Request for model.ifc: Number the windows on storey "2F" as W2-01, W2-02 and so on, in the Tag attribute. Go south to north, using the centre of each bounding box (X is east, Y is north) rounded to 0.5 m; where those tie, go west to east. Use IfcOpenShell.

First a look at what the model holds.

```python
import ifcopenshell
import ifcopenshell.util.element
import ifcopenshell.util.placement

model = ifcopenshell.open("model.ifc")
print(model.schema)
storey = next(s for s in model.by_type("IfcBuildingStorey") if s.Name == "2F")
windows = [e for e in ifcopenshell.util.element.get_decomposition(storey) if e.is_a("IfcWindow")]
for e in sorted(windows, key=lambda e: e.id()):
    origin = ifcopenshell.util.placement.get_local_placement(e.ObjectPlacement)[:3, 3]
    print(e.id(), e.Tag, e.Name, origin.round(2) + 0.0, sep=" | ")
```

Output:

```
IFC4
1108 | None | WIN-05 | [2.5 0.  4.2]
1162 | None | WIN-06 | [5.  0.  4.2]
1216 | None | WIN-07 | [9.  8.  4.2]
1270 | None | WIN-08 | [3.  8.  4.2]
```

```python
import ifcopenshell
import ifcopenshell.geom
import ifcopenshell.util.element
import ifcopenshell.util.shape

model = ifcopenshell.open("model.ifc")
settings = ifcopenshell.geom.settings()
settings.set("use-world-coords", True)


def centre(element):
    shape = ifcopenshell.geom.create_shape(settings, element)
    return ifcopenshell.util.shape.get_bbox_centroid(shape.geometry)


storey = next(s for s in model.by_type("IfcBuildingStorey") if s.Name == "2F")
windows = [e for e in ifcopenshell.util.element.get_decomposition(storey) if e.is_a("IfcWindow")]

# Insertion points can sit at a corner or the storey origin, so sort by the geometry (in metres).
centres = {e: centre(e) for e in windows}
windows.sort(key=lambda e: (round(centres[e][1] / 0.5), centres[e][0]))

for i, e in enumerate(windows, start=1):
    number = f"W2-{i:02d}"
    e.Tag = number
    print(e.id(), number)

model.write("model_rev.ifc")
```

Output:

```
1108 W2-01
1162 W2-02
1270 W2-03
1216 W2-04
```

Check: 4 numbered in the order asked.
